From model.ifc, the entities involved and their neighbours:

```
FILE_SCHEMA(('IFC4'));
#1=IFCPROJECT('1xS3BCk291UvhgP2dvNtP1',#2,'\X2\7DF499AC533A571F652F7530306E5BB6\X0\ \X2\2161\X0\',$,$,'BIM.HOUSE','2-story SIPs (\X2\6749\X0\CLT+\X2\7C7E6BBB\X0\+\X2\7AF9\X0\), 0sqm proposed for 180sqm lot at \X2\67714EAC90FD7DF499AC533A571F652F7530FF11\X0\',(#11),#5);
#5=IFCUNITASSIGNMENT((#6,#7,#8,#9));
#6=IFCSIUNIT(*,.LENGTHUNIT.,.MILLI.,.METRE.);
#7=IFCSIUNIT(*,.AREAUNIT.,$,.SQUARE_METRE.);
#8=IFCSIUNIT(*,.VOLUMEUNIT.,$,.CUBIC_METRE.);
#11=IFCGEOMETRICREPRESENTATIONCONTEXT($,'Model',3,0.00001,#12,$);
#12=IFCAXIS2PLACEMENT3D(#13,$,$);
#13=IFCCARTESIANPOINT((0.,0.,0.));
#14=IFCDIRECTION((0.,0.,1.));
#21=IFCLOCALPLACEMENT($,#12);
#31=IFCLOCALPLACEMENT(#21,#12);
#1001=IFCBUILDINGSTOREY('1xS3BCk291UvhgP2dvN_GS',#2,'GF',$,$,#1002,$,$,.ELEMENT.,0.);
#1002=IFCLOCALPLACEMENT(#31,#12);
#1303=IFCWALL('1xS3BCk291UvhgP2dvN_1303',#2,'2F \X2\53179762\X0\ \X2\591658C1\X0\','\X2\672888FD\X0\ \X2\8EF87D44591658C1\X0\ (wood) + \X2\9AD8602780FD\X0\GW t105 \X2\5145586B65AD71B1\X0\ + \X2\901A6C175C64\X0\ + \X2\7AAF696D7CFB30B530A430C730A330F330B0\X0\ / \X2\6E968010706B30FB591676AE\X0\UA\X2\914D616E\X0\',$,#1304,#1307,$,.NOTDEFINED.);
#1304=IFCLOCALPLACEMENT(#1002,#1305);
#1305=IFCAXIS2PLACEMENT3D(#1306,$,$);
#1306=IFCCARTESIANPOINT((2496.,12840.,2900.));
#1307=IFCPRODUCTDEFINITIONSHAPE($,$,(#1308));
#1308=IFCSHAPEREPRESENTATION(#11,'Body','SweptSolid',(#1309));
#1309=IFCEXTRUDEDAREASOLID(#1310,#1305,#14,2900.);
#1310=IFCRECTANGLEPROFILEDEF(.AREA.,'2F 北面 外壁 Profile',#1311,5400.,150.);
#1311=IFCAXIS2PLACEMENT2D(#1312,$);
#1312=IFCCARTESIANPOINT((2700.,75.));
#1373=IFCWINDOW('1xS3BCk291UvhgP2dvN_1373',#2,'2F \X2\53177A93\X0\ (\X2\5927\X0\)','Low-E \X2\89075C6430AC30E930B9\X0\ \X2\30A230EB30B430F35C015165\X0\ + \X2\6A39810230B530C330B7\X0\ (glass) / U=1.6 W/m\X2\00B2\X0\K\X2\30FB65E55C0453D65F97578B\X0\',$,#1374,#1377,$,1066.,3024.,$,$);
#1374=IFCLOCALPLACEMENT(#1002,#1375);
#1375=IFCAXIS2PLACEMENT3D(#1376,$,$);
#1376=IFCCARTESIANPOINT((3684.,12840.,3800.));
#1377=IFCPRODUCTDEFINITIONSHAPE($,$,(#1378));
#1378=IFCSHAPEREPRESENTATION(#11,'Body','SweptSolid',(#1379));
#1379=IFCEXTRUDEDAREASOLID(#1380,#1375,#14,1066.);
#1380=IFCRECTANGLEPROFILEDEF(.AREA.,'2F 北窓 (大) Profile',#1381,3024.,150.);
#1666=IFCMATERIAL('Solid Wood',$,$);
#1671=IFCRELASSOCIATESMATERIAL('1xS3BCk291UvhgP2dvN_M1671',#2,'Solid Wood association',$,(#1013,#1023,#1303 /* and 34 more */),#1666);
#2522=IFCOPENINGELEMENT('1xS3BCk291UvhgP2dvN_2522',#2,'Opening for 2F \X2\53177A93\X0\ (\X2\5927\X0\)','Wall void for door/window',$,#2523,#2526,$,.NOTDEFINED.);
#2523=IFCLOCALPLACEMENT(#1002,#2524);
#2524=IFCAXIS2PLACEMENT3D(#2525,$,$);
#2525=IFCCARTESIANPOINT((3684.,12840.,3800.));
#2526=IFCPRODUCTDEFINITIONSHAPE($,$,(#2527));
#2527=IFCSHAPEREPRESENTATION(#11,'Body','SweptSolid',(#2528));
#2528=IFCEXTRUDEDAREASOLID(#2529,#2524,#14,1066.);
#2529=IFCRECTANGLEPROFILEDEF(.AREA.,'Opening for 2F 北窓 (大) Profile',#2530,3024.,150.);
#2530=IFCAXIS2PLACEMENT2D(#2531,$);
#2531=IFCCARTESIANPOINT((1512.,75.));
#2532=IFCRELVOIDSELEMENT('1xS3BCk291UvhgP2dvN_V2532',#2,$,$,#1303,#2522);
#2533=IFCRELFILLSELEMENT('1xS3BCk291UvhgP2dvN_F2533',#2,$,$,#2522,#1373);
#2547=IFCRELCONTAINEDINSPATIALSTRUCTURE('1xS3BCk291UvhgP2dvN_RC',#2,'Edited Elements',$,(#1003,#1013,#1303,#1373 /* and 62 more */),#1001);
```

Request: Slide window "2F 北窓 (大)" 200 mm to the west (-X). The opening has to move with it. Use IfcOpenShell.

```python
import ifcopenshell
import ifcopenshell.api.geometry
import ifcopenshell.util.placement

model = ifcopenshell.open("model.ifc")

window = model.by_guid("1xS3BCk291UvhgP2dvN_1373")
opening = window.FillsVoids[0].RelatingOpeningElement
wall = opening.VoidsElements[0].RelatingBuildingElement

wall_matrix = ifcopenshell.util.placement.get_local_placement(wall.ObjectPlacement)
shift = wall_matrix[:3, 0] * -200.0
before = ifcopenshell.util.placement.get_local_placement(window.ObjectPlacement)[:3, 3].copy()

# The window is not placed relative to its opening, so move both.
for product in (opening, window):
    matrix = ifcopenshell.util.placement.get_local_placement(product.ObjectPlacement)
    matrix[:3, 3] += shift
    ifcopenshell.api.geometry.edit_object_placement(model, product=product, matrix=matrix, is_si=False)

after = ifcopenshell.util.placement.get_local_placement(window.ObjectPlacement)[:3, 3]
print("window moved by", (after - before).round(3) + 0.0)

model.write("model_v2.ifc")
```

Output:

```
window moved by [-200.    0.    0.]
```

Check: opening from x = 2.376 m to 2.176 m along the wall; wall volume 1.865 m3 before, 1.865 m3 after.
